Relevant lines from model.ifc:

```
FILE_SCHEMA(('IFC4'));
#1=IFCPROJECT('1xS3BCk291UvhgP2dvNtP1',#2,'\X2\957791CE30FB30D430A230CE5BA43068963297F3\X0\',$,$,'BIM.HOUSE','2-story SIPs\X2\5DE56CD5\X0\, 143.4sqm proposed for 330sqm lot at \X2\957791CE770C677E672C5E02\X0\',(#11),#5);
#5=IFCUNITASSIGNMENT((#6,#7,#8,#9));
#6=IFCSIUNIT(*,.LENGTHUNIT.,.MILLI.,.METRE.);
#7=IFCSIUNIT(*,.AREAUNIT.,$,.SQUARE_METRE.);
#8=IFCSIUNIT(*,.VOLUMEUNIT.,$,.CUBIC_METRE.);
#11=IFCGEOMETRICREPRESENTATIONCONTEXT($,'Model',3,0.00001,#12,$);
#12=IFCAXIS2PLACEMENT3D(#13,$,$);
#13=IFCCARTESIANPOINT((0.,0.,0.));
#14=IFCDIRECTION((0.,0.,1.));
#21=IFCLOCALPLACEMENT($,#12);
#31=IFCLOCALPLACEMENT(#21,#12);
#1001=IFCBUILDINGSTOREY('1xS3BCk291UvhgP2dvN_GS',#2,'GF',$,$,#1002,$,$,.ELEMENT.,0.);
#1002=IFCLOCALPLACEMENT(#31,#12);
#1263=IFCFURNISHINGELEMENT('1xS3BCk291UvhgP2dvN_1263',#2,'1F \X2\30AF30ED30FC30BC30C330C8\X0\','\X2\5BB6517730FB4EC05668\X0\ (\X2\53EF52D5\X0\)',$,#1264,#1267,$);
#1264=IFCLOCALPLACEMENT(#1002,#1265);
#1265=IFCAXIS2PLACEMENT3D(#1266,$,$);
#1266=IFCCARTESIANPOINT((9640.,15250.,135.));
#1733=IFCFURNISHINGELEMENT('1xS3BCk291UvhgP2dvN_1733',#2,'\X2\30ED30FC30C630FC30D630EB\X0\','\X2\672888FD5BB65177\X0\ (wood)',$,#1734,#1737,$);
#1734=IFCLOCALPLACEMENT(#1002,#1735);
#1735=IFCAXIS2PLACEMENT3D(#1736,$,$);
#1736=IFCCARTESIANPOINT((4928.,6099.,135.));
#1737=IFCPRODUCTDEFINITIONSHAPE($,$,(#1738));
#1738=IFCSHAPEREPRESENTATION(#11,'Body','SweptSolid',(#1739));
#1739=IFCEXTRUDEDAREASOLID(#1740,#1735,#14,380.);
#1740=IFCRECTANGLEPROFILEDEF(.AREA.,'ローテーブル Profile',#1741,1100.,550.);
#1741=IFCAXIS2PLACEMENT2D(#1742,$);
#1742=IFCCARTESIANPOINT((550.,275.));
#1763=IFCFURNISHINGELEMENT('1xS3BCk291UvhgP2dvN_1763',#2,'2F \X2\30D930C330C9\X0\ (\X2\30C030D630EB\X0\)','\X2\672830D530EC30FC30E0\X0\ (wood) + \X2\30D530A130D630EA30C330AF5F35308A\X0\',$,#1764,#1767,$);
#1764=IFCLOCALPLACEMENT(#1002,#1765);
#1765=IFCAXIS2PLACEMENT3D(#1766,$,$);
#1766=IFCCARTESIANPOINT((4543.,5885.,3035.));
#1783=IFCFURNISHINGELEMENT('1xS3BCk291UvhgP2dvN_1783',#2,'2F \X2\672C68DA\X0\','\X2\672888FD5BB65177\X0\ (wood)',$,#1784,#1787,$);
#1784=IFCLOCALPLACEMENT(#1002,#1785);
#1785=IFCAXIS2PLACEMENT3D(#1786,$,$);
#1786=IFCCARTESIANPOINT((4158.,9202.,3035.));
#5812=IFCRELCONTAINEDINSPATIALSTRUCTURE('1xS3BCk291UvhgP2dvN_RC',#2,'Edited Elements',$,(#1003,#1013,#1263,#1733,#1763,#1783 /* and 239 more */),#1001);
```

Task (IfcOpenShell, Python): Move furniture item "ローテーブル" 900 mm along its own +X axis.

```python
import ifcopenshell
import ifcopenshell.api.geometry
import ifcopenshell.util.placement
import ifcopenshell.util.unit

model = ifcopenshell.open("model.ifc")
unit_scale = ifcopenshell.util.unit.calculate_unit_scale(model)

item = model.by_guid("1xS3BCk291UvhgP2dvN_1733")
matrix = ifcopenshell.util.placement.get_local_placement(item.ObjectPlacement)
matrix[:3, 3] += matrix[:3, 0] * 0.9 / unit_scale
ifcopenshell.api.geometry.edit_object_placement(model, product=item, matrix=matrix, is_si=False)

print(ifcopenshell.util.placement.get_local_placement(item.ObjectPlacement).round(3) + 0.0)

model.write("model_edited.ifc")
```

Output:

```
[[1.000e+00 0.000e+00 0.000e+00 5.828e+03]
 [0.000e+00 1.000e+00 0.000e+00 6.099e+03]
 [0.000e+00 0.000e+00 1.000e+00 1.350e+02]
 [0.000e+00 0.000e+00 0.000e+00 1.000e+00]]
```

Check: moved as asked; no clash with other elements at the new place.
